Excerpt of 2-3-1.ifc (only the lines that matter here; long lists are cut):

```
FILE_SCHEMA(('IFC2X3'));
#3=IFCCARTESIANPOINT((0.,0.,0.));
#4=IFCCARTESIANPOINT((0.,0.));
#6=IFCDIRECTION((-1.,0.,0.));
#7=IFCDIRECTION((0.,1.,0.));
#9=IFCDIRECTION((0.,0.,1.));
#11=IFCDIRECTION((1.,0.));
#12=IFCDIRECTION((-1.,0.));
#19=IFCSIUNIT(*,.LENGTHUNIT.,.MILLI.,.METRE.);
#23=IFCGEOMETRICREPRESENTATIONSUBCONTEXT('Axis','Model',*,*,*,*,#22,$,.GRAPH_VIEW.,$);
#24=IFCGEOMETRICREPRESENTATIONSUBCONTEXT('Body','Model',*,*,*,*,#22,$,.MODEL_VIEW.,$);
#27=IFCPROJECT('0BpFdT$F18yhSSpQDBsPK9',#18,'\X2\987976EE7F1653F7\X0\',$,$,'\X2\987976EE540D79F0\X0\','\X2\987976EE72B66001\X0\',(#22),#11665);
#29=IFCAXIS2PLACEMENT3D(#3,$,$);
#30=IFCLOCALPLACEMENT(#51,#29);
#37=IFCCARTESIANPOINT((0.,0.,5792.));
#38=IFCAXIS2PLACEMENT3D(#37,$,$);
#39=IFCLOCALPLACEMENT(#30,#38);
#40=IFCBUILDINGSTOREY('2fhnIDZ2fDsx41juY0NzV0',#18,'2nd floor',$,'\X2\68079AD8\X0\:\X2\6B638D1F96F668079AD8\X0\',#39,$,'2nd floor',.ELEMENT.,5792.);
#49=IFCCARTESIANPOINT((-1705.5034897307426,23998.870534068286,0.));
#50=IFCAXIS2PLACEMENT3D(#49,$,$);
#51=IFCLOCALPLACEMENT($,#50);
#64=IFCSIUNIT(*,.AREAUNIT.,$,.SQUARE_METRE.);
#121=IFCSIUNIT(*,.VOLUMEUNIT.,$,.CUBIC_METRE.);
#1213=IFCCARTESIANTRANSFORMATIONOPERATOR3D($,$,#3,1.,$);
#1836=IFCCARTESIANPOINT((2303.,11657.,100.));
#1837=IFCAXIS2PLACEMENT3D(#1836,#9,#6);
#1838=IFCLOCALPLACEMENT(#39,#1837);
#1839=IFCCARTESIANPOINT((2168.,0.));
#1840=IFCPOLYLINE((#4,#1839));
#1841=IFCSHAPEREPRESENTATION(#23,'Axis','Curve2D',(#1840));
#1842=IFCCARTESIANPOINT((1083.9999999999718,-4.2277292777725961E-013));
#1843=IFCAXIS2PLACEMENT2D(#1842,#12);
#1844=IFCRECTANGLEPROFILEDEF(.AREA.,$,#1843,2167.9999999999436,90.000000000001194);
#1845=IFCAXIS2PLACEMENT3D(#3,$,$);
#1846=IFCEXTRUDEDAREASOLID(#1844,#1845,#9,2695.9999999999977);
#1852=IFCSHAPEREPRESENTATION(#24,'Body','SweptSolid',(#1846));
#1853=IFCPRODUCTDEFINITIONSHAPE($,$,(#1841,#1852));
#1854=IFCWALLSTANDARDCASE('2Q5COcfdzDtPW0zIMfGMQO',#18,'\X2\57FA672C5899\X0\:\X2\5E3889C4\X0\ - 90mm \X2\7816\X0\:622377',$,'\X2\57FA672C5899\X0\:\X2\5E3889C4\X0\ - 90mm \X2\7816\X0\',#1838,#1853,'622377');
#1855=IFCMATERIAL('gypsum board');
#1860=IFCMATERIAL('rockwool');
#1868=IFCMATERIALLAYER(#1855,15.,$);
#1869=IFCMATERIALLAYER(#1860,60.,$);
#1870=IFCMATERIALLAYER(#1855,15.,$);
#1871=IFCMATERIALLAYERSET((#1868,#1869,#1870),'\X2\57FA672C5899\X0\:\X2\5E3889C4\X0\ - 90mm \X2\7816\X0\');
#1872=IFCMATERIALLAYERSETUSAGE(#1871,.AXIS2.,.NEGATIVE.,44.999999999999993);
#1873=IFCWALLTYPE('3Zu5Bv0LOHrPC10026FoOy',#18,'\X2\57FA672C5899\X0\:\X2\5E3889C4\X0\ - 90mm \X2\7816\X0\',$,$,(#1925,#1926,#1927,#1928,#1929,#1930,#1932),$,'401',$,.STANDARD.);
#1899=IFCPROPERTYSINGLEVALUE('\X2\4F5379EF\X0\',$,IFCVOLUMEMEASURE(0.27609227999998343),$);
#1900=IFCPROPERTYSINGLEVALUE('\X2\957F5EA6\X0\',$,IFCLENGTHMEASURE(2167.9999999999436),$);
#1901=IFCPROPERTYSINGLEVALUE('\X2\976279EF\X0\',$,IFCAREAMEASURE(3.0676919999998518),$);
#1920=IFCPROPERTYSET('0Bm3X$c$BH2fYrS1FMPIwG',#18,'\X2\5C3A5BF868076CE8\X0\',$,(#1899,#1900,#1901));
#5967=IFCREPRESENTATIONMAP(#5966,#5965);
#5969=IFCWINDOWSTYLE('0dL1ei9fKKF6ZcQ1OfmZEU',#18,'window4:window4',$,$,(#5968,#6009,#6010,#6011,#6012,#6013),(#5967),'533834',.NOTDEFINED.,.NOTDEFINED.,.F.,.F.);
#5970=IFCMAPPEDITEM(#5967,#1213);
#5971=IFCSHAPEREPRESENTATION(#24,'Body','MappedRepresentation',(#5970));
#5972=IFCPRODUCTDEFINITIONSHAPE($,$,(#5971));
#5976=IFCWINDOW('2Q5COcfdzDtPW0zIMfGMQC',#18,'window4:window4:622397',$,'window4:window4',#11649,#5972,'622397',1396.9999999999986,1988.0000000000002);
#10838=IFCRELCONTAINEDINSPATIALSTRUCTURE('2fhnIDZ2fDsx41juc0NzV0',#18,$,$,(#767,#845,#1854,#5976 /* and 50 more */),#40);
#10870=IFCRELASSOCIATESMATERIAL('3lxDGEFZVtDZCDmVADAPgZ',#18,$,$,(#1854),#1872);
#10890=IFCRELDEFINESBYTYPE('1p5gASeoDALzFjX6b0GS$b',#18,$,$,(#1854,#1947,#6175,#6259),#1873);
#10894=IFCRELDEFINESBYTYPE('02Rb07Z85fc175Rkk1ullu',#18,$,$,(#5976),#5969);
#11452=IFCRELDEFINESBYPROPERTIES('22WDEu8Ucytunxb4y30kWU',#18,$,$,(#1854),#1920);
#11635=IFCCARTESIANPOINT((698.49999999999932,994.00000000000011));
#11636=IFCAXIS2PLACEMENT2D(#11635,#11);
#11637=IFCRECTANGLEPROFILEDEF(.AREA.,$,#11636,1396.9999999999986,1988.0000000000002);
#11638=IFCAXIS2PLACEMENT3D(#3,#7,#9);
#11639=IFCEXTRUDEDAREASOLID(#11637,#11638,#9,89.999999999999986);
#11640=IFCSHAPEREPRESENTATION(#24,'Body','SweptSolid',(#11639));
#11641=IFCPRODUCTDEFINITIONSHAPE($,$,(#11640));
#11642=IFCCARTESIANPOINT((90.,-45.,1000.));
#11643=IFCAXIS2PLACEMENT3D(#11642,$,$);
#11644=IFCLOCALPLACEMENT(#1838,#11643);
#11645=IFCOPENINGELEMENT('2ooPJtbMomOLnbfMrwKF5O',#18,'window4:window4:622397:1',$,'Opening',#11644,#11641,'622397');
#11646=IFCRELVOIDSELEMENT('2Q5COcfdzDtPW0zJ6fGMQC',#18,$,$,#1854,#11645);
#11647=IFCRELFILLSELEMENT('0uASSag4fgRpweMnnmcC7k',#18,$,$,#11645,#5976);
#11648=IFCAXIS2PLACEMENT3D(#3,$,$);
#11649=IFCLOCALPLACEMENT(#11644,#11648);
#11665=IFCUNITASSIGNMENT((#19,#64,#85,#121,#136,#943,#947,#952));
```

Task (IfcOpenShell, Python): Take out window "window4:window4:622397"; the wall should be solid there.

```python
import ifcopenshell
import ifcopenshell.api.feature
import ifcopenshell.api.pset
import ifcopenshell.api.root
import ifcopenshell.geom
import ifcopenshell.util.element
import ifcopenshell.util.shape
import ifcopenshell.util.unit

model = ifcopenshell.open("2-3-1.ifc")
area_scale = ifcopenshell.util.unit.calculate_unit_scale(model, "AREAUNIT")
volume_scale = ifcopenshell.util.unit.calculate_unit_scale(model, "VOLUMEUNIT")
settings = ifcopenshell.geom.settings()


def volume(element):
    """Net volume in cubic metres, openings subtracted."""
    shape = ifcopenshell.geom.create_shape(settings, element)
    return ifcopenshell.util.shape.get_volume(shape.geometry)


window = model.by_id(5976)
opening = window.FillsVoids[0].RelatingOpeningElement
wall = opening.VoidsElements[0].RelatingBuildingElement
before = volume(wall)

ifcopenshell.api.root.remove_product(model, product=window)
ifcopenshell.api.feature.remove_feature(model, feature=opening)

after = volume(wall)
thickness = 0.09  # wall thickness in metres

# Update the wall's stored quantities.
pset = model.by_id(ifcopenshell.util.element.get_pset(wall, "尺寸标注", should_inherit=False)["id"])
ifcopenshell.api.pset.edit_pset(model, pset=pset, properties={
    "体积": model.create_entity("IfcVolumeMeasure", after / volume_scale),
    "面积": model.create_entity("IfcAreaMeasure", after / thickness / area_scale),
})

print(f"wall volume {before:.3f} -> {after:.3f} m3")

model.write("2-3-1_edited.ifc")
```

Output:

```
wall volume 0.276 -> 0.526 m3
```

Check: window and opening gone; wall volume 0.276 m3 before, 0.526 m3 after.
